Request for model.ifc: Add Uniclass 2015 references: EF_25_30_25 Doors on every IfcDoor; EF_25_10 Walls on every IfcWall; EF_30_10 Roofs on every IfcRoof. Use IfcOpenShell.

First a look at what the model holds.

```python
import ifcopenshell

model = ifcopenshell.open("model.ifc")
print(model.schema)
print("classifications:", [c.Name for c in model.by_type("IfcClassification")])
for ifc_class in ("IfcDoor", "IfcRoof", "IfcStair", "IfcWall", "IfcWindow"):
    print(ifc_class, len(model.by_type(ifc_class)))
```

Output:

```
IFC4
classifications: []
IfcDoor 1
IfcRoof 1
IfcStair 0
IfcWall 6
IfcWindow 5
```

```python
import ifcopenshell
import ifcopenshell.api.classification

model = ifcopenshell.open("model.ifc")

system = ifcopenshell.api.classification.add_classification(model, classification="Uniclass 2015")

codes = {
    "IfcDoor": ("EF_25_30_25", "Doors"),
    "IfcWall": ("EF_25_10", "Walls"),
    "IfcRoof": ("EF_30_10", "Roofs"),
}
for ifc_class, (code, name) in codes.items():
    products = model.by_type(ifc_class)
    ifcopenshell.api.classification.add_reference(
        model, products=products, classification=system, identification=code, name=name
    )
    print(code, len(products))

model.write("model_rev.ifc")
```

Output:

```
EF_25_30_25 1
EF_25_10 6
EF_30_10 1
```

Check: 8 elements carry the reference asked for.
